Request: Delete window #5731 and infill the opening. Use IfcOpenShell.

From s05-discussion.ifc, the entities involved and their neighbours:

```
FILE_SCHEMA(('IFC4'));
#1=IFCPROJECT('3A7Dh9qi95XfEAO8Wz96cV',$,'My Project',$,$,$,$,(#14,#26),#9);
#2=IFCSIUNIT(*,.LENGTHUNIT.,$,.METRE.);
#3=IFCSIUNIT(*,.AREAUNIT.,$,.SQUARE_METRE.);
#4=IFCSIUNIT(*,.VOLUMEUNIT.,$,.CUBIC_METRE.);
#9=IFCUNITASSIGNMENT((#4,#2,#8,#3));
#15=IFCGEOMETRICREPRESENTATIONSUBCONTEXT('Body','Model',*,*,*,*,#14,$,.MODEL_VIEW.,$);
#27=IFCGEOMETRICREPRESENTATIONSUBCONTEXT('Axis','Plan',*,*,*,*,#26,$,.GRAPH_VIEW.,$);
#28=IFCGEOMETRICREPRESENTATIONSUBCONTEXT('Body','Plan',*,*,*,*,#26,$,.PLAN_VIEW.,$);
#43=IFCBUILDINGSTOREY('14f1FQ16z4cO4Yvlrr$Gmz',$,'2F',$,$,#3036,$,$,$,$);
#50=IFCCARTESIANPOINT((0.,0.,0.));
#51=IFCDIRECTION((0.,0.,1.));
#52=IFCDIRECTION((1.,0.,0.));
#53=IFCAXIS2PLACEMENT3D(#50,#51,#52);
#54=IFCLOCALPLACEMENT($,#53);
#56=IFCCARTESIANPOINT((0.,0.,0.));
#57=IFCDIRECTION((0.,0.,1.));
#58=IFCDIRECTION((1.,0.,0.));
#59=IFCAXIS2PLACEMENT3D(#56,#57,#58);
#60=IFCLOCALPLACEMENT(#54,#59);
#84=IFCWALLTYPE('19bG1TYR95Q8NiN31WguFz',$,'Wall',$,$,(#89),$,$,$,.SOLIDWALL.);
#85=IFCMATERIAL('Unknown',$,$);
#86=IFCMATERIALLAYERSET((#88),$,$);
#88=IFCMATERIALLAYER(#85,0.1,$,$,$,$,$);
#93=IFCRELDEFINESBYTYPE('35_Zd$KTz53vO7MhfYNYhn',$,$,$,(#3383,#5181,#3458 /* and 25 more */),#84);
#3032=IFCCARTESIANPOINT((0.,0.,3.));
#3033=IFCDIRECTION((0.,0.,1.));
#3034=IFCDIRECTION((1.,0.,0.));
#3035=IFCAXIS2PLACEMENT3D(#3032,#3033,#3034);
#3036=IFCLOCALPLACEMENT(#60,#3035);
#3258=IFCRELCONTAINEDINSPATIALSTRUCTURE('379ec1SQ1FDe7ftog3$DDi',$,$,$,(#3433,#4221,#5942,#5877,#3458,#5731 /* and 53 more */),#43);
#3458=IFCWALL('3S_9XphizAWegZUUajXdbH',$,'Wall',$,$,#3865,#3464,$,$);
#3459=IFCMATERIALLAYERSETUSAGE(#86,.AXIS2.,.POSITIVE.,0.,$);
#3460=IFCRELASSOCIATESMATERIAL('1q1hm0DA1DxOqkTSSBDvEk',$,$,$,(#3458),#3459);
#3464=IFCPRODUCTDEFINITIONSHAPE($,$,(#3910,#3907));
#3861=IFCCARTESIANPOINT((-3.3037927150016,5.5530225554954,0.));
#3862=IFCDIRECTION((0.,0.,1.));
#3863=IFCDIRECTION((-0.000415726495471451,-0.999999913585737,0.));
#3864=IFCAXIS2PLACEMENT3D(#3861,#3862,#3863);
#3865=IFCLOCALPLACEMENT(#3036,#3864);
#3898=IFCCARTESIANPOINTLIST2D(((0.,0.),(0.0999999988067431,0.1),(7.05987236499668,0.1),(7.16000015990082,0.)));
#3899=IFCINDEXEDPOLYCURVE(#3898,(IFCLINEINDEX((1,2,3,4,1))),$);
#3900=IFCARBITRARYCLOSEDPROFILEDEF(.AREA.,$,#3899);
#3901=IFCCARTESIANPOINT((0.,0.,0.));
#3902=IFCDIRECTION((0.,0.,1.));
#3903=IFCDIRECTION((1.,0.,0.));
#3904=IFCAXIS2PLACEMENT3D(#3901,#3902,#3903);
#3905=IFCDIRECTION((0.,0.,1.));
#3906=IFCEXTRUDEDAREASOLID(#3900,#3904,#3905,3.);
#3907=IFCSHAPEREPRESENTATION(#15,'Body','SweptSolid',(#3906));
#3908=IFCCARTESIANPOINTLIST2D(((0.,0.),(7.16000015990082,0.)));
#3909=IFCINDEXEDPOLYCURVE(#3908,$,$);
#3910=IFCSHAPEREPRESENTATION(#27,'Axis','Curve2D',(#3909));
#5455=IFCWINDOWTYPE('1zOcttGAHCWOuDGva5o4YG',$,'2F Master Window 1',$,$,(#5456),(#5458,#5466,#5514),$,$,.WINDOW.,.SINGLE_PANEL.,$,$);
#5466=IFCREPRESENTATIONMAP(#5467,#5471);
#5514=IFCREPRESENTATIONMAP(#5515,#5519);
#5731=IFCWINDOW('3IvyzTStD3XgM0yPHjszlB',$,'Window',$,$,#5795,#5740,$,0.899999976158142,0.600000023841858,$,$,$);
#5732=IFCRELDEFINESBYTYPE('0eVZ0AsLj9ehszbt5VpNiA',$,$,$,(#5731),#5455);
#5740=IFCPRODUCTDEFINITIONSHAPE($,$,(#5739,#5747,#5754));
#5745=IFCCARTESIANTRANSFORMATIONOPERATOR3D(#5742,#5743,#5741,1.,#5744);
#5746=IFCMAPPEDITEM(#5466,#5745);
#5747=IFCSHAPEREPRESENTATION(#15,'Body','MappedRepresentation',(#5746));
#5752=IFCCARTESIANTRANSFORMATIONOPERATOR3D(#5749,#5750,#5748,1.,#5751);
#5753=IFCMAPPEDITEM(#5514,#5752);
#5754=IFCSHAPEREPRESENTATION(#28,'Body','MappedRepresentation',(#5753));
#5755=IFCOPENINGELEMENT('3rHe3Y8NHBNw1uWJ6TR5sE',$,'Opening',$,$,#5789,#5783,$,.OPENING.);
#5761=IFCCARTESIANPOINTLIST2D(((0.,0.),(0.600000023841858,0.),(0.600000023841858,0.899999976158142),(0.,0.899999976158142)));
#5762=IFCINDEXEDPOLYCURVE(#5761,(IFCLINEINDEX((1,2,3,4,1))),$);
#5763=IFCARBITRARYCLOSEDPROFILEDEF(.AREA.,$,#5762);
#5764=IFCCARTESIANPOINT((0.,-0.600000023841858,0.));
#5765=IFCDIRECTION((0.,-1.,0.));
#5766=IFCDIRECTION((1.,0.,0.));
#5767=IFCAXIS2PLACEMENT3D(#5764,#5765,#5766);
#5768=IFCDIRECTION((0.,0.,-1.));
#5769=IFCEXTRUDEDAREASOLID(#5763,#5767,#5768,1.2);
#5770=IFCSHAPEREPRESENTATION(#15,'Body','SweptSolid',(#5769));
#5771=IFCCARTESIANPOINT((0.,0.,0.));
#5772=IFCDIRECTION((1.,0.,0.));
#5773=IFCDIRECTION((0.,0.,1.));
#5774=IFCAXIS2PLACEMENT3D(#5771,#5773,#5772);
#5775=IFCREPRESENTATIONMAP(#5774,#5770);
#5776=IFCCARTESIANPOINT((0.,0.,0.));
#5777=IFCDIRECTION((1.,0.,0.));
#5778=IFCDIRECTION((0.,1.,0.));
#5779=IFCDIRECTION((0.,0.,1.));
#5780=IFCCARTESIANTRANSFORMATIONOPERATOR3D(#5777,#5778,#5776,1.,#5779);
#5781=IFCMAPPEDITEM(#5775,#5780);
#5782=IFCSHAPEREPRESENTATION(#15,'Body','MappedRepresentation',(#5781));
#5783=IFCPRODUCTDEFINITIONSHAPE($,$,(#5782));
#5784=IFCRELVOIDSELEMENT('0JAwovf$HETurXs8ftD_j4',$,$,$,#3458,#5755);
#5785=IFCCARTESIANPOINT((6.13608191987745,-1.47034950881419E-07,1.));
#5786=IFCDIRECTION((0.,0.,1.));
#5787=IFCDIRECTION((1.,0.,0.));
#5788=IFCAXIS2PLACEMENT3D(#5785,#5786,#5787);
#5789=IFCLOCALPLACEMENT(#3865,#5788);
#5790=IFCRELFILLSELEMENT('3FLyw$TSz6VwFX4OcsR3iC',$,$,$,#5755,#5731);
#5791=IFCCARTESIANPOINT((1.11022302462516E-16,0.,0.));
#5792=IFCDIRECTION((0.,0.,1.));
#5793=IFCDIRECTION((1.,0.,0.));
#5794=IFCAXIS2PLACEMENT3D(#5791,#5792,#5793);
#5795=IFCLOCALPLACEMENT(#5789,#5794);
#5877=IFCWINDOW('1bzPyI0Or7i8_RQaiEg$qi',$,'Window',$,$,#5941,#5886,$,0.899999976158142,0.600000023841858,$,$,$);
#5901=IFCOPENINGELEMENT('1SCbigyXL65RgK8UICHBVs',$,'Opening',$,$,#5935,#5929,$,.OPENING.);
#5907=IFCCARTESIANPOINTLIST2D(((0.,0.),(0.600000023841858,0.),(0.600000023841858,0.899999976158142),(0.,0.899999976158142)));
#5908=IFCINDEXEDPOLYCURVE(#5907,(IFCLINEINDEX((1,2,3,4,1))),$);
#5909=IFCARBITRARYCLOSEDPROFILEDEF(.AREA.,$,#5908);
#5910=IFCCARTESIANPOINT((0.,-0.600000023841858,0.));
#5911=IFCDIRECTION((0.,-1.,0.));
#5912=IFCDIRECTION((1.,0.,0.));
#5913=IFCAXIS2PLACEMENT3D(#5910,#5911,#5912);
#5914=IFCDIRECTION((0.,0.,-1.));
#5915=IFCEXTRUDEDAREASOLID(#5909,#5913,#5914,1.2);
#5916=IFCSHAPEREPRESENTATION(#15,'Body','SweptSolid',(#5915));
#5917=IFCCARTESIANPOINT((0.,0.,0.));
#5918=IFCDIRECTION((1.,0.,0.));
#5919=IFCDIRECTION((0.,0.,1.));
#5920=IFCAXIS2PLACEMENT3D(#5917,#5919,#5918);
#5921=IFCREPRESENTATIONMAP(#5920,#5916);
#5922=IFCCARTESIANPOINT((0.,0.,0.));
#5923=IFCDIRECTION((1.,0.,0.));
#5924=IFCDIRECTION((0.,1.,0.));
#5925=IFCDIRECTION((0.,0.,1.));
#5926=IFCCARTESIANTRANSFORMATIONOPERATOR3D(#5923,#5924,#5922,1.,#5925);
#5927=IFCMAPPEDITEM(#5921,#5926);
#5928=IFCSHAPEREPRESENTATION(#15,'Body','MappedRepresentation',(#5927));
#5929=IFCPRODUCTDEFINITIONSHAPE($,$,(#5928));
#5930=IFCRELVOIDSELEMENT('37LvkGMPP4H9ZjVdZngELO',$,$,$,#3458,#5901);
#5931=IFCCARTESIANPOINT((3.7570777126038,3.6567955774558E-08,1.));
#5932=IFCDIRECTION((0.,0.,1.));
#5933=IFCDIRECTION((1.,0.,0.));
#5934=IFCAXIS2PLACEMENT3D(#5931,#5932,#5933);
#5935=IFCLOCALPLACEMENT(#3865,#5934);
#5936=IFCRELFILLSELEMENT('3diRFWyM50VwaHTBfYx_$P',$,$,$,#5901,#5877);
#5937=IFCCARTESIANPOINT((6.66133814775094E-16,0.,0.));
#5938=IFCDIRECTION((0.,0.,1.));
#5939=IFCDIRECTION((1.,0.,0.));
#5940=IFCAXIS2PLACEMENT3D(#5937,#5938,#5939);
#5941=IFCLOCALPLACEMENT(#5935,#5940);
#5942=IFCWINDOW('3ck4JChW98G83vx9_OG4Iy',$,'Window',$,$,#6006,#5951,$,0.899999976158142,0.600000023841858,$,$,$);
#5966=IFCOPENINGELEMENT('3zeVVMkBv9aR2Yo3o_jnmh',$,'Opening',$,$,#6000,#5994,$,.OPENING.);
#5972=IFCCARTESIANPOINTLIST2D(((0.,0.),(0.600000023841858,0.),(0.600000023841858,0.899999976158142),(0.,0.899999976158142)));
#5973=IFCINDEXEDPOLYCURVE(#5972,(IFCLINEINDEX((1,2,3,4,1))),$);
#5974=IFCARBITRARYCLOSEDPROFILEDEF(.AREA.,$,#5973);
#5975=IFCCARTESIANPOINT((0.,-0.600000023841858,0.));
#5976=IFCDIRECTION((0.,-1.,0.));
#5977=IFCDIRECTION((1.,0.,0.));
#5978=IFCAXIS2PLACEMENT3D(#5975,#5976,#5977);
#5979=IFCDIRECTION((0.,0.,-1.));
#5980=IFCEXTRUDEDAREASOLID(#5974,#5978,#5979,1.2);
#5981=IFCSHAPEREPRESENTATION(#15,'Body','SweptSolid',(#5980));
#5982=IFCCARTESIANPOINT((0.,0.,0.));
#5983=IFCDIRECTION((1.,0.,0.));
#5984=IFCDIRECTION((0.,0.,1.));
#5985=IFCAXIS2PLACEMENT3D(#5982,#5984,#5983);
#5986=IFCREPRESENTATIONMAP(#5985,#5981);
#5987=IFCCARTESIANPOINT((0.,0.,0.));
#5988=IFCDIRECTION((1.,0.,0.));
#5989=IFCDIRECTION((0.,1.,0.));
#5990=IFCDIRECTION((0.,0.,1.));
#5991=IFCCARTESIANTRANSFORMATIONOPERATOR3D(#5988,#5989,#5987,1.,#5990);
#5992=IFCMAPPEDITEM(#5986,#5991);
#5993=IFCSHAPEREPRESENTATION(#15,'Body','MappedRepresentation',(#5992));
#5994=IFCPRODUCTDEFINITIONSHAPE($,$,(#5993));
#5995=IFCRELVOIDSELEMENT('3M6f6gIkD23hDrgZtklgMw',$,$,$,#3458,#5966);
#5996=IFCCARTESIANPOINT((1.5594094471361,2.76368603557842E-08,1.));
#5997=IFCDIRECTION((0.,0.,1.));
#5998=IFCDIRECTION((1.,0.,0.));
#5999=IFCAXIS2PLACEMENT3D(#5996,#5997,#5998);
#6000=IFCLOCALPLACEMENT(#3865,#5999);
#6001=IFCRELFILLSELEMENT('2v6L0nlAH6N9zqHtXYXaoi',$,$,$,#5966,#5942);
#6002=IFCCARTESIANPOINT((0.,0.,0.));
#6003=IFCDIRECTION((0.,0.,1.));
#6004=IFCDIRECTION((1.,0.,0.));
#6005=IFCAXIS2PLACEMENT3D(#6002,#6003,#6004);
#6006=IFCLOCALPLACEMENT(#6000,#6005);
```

```python
import ifcopenshell
import ifcopenshell.api.feature
import ifcopenshell.api.root
import ifcopenshell.geom
import ifcopenshell.util.shape

model = ifcopenshell.open("s05-discussion.ifc")
settings = ifcopenshell.geom.settings()


def volume(element):
    """Net volume in cubic metres, openings subtracted."""
    shape = ifcopenshell.geom.create_shape(settings, element)
    return ifcopenshell.util.shape.get_volume(shape.geometry)


window = model.by_id(5731)
opening = window.FillsVoids[0].RelatingOpeningElement
wall = opening.VoidsElements[0].RelatingBuildingElement
before = volume(wall)

ifcopenshell.api.root.remove_product(model, product=window)
ifcopenshell.api.feature.remove_feature(model, feature=opening)

after = volume(wall)

print(f"wall volume {before:.3f} -> {after:.3f} m3")

model.write("s05-discussion_updated.ifc")
```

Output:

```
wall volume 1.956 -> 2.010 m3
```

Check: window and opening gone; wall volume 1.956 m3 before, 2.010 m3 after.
